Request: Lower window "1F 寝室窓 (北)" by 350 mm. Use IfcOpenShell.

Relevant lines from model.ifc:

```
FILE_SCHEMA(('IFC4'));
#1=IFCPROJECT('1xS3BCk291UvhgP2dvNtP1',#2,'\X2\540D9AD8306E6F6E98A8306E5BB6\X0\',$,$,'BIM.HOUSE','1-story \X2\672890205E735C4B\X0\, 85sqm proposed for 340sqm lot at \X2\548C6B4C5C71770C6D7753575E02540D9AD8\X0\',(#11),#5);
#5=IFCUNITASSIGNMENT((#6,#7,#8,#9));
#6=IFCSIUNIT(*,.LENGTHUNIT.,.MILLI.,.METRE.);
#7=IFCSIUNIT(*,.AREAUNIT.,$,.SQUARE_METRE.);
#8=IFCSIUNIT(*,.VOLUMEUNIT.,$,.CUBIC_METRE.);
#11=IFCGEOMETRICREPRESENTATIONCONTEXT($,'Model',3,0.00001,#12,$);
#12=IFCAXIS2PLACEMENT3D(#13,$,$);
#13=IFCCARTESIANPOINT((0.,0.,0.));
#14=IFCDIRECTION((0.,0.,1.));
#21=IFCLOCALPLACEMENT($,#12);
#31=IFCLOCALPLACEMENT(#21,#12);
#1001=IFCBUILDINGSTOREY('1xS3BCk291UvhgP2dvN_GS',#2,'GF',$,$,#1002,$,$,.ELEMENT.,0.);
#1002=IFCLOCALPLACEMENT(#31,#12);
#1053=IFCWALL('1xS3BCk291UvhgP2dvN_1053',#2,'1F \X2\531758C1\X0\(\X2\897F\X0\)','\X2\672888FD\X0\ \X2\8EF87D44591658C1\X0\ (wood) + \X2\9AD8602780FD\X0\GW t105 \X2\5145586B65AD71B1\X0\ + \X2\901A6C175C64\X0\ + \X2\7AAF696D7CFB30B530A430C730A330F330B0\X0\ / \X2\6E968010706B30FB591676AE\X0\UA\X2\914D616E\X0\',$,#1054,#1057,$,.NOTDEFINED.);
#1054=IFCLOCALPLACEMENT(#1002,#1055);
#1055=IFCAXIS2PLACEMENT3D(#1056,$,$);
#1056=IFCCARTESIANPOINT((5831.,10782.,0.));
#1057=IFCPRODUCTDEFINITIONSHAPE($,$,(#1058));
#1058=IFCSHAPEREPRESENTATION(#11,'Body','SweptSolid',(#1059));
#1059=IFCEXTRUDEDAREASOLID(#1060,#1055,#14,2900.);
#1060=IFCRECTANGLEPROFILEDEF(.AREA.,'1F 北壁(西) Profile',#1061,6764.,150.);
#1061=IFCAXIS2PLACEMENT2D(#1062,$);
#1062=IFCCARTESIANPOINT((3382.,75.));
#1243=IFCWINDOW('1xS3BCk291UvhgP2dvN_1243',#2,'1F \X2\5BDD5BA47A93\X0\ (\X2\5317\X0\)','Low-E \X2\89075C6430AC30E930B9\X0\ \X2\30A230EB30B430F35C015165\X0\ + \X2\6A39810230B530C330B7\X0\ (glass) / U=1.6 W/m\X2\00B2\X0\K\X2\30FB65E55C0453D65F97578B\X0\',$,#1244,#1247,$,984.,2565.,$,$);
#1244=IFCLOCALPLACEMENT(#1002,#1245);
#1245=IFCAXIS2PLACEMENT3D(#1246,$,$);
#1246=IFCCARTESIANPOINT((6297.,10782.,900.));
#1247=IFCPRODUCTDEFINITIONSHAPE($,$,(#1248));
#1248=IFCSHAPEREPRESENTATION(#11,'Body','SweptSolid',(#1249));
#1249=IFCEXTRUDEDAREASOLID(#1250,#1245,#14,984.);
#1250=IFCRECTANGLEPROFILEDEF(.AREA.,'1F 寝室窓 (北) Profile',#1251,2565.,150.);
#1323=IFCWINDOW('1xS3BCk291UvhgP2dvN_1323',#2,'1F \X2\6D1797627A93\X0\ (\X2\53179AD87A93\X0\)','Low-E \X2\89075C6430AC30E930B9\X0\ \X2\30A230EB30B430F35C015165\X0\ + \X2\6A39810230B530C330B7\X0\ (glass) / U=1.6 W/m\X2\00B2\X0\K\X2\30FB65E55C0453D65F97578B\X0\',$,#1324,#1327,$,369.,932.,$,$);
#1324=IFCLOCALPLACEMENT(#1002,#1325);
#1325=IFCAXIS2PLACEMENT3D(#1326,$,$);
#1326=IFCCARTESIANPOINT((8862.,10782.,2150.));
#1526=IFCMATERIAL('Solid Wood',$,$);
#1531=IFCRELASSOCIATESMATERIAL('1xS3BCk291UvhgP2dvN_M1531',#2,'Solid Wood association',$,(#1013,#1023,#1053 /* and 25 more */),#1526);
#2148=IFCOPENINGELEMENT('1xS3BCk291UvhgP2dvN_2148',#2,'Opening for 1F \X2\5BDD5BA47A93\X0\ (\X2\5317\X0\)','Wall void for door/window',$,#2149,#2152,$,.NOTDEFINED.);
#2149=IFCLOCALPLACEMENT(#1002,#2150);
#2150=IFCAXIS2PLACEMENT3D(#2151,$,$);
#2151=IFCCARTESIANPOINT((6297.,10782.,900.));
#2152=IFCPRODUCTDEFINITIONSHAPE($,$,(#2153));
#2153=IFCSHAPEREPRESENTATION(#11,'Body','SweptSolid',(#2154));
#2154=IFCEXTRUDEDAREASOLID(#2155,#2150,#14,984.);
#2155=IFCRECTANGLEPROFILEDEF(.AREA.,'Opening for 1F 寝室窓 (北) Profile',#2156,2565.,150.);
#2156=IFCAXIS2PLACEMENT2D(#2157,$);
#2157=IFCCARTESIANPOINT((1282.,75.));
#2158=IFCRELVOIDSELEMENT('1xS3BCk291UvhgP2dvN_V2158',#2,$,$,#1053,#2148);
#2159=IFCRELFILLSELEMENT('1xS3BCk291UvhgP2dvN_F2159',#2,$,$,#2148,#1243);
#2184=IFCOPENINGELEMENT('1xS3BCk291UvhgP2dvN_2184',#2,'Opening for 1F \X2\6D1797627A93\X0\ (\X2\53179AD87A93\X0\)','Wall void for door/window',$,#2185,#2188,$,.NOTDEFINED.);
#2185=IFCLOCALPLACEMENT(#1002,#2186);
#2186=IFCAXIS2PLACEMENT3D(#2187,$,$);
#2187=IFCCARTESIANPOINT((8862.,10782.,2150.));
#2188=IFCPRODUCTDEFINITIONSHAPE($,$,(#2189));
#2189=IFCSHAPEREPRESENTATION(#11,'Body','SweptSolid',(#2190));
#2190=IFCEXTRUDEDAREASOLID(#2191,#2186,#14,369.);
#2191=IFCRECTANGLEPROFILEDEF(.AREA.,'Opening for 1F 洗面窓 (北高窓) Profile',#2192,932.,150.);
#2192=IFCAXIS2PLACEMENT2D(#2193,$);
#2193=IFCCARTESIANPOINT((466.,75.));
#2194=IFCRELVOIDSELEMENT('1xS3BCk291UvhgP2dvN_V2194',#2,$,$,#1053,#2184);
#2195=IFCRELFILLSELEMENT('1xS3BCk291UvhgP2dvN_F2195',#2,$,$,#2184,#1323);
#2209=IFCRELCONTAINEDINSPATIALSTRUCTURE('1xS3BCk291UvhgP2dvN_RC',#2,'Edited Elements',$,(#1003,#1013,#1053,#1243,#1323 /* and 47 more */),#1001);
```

```python
import numpy as np
import ifcopenshell
import ifcopenshell.api.geometry
import ifcopenshell.util.placement
import ifcopenshell.util.unit

model = ifcopenshell.open("model.ifc")
unit_scale = ifcopenshell.util.unit.calculate_unit_scale(model)

window = model.by_guid("1xS3BCk291UvhgP2dvN_1243")
opening = window.FillsVoids[0].RelatingOpeningElement
dz = -350.0

shift = np.array([0.0, 0.0, dz])
# The window is not placed relative to its opening, so move both.
for product in (opening, window):
    matrix = ifcopenshell.util.placement.get_local_placement(product.ObjectPlacement)
    matrix[:3, 3] += shift
    ifcopenshell.api.geometry.edit_object_placement(model, product=product, matrix=matrix, is_si=False)

print(f"moved by {dz * unit_scale:+.3f} m")

model.write("model_updated.ifc")
```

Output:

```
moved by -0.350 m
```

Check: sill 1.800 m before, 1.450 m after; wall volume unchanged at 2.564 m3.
